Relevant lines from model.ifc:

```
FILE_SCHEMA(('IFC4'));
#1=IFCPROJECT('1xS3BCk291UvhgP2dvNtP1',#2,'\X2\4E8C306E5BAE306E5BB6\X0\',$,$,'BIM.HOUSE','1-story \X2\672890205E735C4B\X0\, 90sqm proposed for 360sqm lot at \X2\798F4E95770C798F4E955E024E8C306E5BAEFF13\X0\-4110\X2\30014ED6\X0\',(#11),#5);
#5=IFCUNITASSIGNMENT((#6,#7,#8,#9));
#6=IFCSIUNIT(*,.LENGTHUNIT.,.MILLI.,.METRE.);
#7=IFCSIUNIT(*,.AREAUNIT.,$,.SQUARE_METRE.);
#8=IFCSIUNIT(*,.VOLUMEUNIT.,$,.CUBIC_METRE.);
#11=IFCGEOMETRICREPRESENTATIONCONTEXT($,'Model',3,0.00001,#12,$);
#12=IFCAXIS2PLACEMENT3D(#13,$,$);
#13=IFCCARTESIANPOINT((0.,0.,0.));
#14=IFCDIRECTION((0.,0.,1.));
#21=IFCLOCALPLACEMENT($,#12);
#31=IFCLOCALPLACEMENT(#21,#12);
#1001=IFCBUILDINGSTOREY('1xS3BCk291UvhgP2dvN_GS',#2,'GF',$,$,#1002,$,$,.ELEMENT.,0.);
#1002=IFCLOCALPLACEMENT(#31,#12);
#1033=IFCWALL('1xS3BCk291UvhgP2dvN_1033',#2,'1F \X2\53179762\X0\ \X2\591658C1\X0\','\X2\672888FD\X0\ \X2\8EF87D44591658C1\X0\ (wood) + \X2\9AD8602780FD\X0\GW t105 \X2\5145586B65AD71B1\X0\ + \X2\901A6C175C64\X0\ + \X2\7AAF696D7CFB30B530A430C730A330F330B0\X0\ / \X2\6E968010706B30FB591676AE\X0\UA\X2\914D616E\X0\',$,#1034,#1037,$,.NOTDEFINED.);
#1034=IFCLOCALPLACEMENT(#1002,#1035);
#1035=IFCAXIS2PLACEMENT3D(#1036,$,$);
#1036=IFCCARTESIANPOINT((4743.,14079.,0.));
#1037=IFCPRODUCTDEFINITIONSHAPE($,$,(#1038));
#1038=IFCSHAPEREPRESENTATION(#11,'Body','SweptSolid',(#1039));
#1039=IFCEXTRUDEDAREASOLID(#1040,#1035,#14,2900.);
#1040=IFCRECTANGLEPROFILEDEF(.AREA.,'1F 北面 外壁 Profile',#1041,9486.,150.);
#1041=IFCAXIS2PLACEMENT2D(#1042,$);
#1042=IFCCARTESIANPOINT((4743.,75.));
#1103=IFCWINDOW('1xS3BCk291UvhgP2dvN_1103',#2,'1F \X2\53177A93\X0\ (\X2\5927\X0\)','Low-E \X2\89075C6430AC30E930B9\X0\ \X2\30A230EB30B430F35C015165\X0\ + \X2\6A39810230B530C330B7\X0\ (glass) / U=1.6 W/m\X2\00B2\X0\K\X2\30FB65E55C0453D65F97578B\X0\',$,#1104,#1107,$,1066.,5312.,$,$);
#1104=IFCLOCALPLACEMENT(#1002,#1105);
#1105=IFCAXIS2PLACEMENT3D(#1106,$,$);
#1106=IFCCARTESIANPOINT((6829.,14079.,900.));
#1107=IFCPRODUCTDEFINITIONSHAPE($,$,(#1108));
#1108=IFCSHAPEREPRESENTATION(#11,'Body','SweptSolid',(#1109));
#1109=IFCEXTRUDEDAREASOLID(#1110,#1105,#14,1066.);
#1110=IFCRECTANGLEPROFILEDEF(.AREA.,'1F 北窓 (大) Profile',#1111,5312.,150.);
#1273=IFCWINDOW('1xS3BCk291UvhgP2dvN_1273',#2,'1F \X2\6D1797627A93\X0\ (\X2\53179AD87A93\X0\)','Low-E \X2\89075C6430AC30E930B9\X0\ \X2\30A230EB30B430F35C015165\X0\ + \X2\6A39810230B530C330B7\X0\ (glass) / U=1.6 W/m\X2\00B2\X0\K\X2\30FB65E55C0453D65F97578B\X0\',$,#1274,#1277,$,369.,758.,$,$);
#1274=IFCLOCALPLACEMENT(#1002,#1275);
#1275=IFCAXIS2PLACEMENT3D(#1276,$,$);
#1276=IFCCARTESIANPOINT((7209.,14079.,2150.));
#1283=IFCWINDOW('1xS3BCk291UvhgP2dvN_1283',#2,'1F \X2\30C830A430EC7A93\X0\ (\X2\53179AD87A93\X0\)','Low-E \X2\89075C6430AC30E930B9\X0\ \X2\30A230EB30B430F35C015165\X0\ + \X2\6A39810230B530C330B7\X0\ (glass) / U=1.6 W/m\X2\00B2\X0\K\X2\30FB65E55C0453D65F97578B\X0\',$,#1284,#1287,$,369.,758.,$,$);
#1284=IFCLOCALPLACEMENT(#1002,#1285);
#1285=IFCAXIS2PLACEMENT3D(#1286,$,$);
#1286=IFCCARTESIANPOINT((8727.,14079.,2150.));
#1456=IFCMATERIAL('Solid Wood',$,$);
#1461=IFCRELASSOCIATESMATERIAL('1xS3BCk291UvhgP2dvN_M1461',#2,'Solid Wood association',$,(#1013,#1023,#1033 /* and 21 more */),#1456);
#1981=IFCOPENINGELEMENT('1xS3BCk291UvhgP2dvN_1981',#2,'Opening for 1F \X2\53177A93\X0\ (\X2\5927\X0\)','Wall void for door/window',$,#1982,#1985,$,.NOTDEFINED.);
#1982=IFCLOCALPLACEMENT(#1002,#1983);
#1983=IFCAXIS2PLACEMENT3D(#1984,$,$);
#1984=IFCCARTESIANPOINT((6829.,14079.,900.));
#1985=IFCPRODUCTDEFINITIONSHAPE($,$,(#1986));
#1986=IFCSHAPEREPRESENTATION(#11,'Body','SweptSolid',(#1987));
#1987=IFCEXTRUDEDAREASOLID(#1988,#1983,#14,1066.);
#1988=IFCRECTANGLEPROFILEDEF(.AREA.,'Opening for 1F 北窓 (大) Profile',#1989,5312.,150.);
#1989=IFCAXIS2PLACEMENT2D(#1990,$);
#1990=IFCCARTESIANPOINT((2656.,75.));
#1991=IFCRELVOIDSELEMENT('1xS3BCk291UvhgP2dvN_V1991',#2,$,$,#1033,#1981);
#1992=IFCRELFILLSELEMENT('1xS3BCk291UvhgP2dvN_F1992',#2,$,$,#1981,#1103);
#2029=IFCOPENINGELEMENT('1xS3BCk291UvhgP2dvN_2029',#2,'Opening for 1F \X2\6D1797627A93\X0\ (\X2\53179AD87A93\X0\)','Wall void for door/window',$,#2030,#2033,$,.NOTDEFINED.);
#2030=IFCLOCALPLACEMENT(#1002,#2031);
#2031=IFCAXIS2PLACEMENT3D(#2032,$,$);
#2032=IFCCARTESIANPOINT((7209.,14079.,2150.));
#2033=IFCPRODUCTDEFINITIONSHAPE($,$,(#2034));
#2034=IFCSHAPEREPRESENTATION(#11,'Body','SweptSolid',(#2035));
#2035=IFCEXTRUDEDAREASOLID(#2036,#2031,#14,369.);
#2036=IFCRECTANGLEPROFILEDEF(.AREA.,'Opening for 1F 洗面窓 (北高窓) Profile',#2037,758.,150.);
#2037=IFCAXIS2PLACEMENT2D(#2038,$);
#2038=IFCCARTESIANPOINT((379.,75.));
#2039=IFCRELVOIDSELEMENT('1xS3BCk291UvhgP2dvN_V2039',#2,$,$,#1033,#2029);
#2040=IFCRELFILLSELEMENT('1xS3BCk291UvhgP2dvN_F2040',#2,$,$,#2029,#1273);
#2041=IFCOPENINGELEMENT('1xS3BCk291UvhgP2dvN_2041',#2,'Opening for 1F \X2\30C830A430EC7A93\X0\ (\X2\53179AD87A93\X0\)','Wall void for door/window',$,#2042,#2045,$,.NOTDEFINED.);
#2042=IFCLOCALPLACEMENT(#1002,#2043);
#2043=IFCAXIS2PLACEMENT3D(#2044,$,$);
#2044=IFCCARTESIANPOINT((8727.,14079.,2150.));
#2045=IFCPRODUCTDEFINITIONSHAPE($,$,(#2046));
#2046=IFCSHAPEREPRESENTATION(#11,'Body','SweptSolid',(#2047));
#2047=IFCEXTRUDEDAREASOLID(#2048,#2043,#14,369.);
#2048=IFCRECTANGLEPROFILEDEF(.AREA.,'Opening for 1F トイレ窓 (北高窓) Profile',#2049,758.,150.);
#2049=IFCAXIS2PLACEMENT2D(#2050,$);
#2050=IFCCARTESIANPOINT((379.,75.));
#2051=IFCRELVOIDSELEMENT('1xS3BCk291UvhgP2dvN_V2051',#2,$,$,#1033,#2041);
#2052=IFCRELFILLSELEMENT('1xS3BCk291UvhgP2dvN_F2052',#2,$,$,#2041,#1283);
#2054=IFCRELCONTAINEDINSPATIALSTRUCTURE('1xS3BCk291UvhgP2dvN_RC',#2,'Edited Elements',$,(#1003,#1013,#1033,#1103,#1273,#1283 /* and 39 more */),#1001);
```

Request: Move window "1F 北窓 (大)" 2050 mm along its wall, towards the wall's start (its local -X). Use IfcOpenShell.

```python
import ifcopenshell
import ifcopenshell.api.geometry
import ifcopenshell.util.placement

model = ifcopenshell.open("model.ifc")

window = model.by_guid("1xS3BCk291UvhgP2dvN_1103")
opening = window.FillsVoids[0].RelatingOpeningElement
wall = opening.VoidsElements[0].RelatingBuildingElement

wall_matrix = ifcopenshell.util.placement.get_local_placement(wall.ObjectPlacement)
shift = wall_matrix[:3, 0] * -2050.0
before = ifcopenshell.util.placement.get_local_placement(window.ObjectPlacement)[:3, 3].copy()

# The window is not placed relative to its opening, so move both.
for product in (opening, window):
    matrix = ifcopenshell.util.placement.get_local_placement(product.ObjectPlacement)
    matrix[:3, 3] += shift
    ifcopenshell.api.geometry.edit_object_placement(model, product=product, matrix=matrix, is_si=False)

after = ifcopenshell.util.placement.get_local_placement(window.ObjectPlacement)[:3, 3]
print("window moved by", (after - before).round(3) + 0.0)

model.write("model-out.ifc")
```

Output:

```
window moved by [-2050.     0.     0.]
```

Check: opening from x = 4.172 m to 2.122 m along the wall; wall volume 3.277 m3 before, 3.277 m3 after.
